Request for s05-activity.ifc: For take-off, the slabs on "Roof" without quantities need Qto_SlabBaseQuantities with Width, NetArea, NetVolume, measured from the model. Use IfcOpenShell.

First a look at what the model holds.

```python
import ifcopenshell
import ifcopenshell.util.element
import ifcopenshell.util.unit

model = ifcopenshell.open("s05-activity.ifc")
print(model.schema)
for unit_type in ("LENGTHUNIT", "AREAUNIT", "VOLUMEUNIT"):
    print(unit_type, ifcopenshell.util.unit.calculate_unit_scale(model, unit_type))
storey = next(s for s in model.by_type("IfcBuildingStorey") if s.Name == "Roof")
slabs = [e for e in ifcopenshell.util.element.get_decomposition(storey) if e.is_a("IfcSlab")]
for e in sorted(slabs, key=lambda e: e.id()):
    print(e.id(), e.is_a(), e.Name, list(ifcopenshell.util.element.get_psets(e, qtos_only=True)), sep=" | ")
```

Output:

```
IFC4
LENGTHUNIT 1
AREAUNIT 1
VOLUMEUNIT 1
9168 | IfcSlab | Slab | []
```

```python
import ifcopenshell
import ifcopenshell.api.pset
import ifcopenshell.geom
import ifcopenshell.util.element
import ifcopenshell.util.shape
import ifcopenshell.util.unit

model = ifcopenshell.open("s05-activity.ifc")
unit_scale = ifcopenshell.util.unit.calculate_unit_scale(model)
area_scale = ifcopenshell.util.unit.calculate_unit_scale(model, "AREAUNIT")
volume_scale = ifcopenshell.util.unit.calculate_unit_scale(model, "VOLUMEUNIT")
settings = ifcopenshell.geom.settings()

storey = next(s for s in model.by_type("IfcBuildingStorey") if s.Name == "Roof")
slabs = [e for e in ifcopenshell.util.element.get_decomposition(storey) if e.is_a("IfcSlab")]

for e in sorted(slabs, key=lambda e: e.id()):
    if ifcopenshell.util.element.get_psets(e, qtos_only=True, should_inherit=False):
        continue
    # Geometry comes back in metres, in the element's own axes.
    shape = ifcopenshell.geom.create_shape(settings, e)
    values = {
        "Width": ifcopenshell.util.shape.get_z(shape.geometry) / unit_scale,
        "NetArea": ifcopenshell.util.shape.get_footprint_area(shape.geometry) / area_scale,
        "NetVolume": ifcopenshell.util.shape.get_volume(shape.geometry) / volume_scale,
    }
    qto = ifcopenshell.api.pset.add_qto(model, product=e, name="Qto_SlabBaseQuantities")
    ifcopenshell.api.pset.edit_qto(model, qto=qto, properties=values)
    print(e.id(), {k: round(v, 3) for k, v in values.items()})

model.write("s05-activity_v2.ifc")
```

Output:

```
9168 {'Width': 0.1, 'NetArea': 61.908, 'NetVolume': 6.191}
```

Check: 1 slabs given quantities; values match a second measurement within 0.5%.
